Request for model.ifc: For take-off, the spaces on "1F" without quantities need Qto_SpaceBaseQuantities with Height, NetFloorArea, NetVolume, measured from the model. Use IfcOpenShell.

First a look at what the model holds.

```python
import ifcopenshell
import ifcopenshell.util.element
import ifcopenshell.util.unit

model = ifcopenshell.open("model.ifc")
print(model.schema)
for unit_type in ("LENGTHUNIT", "AREAUNIT", "VOLUMEUNIT"):
    print(unit_type, ifcopenshell.util.unit.calculate_unit_scale(model, unit_type))
storey = next(s for s in model.by_type("IfcBuildingStorey") if s.Name == "1F")
spaces = [e for e in ifcopenshell.util.element.get_decomposition(storey) if e.is_a("IfcSpace")]
for e in sorted(spaces, key=lambda e: e.id()):
    print(e.id(), e.is_a(), e.Name, list(ifcopenshell.util.element.get_psets(e, qtos_only=True)), sep=" | ")
```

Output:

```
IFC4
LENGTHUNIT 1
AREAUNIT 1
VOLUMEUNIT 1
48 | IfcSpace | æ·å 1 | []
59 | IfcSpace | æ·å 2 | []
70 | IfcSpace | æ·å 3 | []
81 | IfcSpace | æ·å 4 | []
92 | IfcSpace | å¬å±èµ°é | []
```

```python
import ifcopenshell
import ifcopenshell.api.pset
import ifcopenshell.geom
import ifcopenshell.util.element
import ifcopenshell.util.shape
import ifcopenshell.util.unit

model = ifcopenshell.open("model.ifc")
unit_scale = ifcopenshell.util.unit.calculate_unit_scale(model)
area_scale = ifcopenshell.util.unit.calculate_unit_scale(model, "AREAUNIT")
volume_scale = ifcopenshell.util.unit.calculate_unit_scale(model, "VOLUMEUNIT")
settings = ifcopenshell.geom.settings()

storey = next(s for s in model.by_type("IfcBuildingStorey") if s.Name == "1F")
spaces = [e for e in ifcopenshell.util.element.get_decomposition(storey) if e.is_a("IfcSpace")]

for e in sorted(spaces, key=lambda e: e.id()):
    if ifcopenshell.util.element.get_psets(e, qtos_only=True, should_inherit=False):
        continue
    # Geometry comes back in metres, in the element's own axes.
    shape = ifcopenshell.geom.create_shape(settings, e)
    values = {
        "Height": ifcopenshell.util.shape.get_z(shape.geometry) / unit_scale,
        "NetFloorArea": ifcopenshell.util.shape.get_footprint_area(shape.geometry) / area_scale,
        "NetVolume": ifcopenshell.util.shape.get_volume(shape.geometry) / volume_scale,
    }
    qto = ifcopenshell.api.pset.add_qto(model, product=e, name="Qto_SpaceBaseQuantities")
    ifcopenshell.api.pset.edit_qto(model, qto=qto, properties=values)
    print(e.id(), {k: round(v, 3) for k, v in values.items()})

model.write("model_edited.ifc")
```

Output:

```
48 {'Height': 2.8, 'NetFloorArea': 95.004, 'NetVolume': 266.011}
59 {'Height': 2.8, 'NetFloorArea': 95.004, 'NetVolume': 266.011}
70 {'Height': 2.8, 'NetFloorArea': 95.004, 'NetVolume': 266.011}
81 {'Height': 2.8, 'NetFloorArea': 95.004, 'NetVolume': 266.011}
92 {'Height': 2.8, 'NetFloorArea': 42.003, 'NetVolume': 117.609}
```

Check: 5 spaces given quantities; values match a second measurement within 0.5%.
